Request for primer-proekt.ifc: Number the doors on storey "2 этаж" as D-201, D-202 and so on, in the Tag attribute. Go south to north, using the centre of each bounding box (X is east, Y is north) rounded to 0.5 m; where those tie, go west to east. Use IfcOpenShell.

First a look at what the model holds.

```python
import ifcopenshell
import ifcopenshell.util.element
import ifcopenshell.util.placement

model = ifcopenshell.open("primer-proekt.ifc")
print(model.schema)
storey = next(s for s in model.by_type("IfcBuildingStorey") if s.Name == "2 этаж")
doors = [e for e in ifcopenshell.util.element.get_decomposition(storey) if e.is_a("IfcDoor")]
for e in sorted(doors, key=lambda e: e.id()):
    origin = ifcopenshell.util.placement.get_local_placement(e.ObjectPlacement)[:3, 3]
    print(e.id(), e.Tag, e.Name, origin.round(2) + 0.0, sep=" | ")
```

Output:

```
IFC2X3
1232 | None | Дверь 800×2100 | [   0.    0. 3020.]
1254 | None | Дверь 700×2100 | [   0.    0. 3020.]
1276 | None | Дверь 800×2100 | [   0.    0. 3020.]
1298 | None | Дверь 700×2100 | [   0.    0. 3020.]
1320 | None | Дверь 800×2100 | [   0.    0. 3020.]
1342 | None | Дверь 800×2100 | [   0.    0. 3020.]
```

```python
import ifcopenshell
import ifcopenshell.geom
import ifcopenshell.util.element
import ifcopenshell.util.shape

model = ifcopenshell.open("primer-proekt.ifc")
settings = ifcopenshell.geom.settings()
settings.set("use-world-coords", True)


def centre(element):
    shape = ifcopenshell.geom.create_shape(settings, element)
    return ifcopenshell.util.shape.get_bbox_centroid(shape.geometry)


storey = next(s for s in model.by_type("IfcBuildingStorey") if s.Name == "2 этаж")
doors = [e for e in ifcopenshell.util.element.get_decomposition(storey) if e.is_a("IfcDoor")]

# Insertion points can sit at a corner or the storey origin, so sort by the geometry (in metres).
centres = {e: centre(e) for e in doors}
doors.sort(key=lambda e: (round(centres[e][1] / 0.5), centres[e][0]))

for i, e in enumerate(doors, start=1):
    number = f"D-2{i:02d}"
    e.Tag = number
    print(e.id(), number)

model.write("primer-proekt_edited.ifc")
```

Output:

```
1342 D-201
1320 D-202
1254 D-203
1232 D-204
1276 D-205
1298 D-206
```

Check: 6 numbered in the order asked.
